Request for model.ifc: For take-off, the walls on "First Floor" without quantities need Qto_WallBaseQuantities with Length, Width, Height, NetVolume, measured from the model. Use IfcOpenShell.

First a look at what the model holds.

```python
import ifcopenshell
import ifcopenshell.util.element
import ifcopenshell.util.unit

model = ifcopenshell.open("model.ifc")
print(model.schema)
for unit_type in ("LENGTHUNIT", "AREAUNIT", "VOLUMEUNIT"):
    print(unit_type, ifcopenshell.util.unit.calculate_unit_scale(model, unit_type))
storey = next(s for s in model.by_type("IfcBuildingStorey") if s.Name == "First Floor")
walls = [e for e in ifcopenshell.util.element.get_decomposition(storey) if e.is_a("IfcWall")]
for e in sorted(walls, key=lambda e: e.id()):
    print(e.id(), e.is_a(), e.Name, list(ifcopenshell.util.element.get_psets(e, qtos_only=True)), sep=" | ")
```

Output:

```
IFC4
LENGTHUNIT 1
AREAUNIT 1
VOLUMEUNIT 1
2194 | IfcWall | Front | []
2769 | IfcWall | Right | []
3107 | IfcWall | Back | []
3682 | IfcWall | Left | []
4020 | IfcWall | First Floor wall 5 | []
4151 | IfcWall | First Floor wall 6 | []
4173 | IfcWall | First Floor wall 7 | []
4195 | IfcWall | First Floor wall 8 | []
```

```python
import ifcopenshell
import ifcopenshell.api.pset
import ifcopenshell.geom
import ifcopenshell.util.element
import ifcopenshell.util.shape
import ifcopenshell.util.unit

model = ifcopenshell.open("model.ifc")
unit_scale = ifcopenshell.util.unit.calculate_unit_scale(model)
volume_scale = ifcopenshell.util.unit.calculate_unit_scale(model, "VOLUMEUNIT")
settings = ifcopenshell.geom.settings()

storey = next(s for s in model.by_type("IfcBuildingStorey") if s.Name == "First Floor")
walls = [e for e in ifcopenshell.util.element.get_decomposition(storey) if e.is_a("IfcWall")]

for e in sorted(walls, key=lambda e: e.id()):
    if ifcopenshell.util.element.get_psets(e, qtos_only=True, should_inherit=False):
        continue
    # Geometry comes back in metres, in the element's own axes.
    shape = ifcopenshell.geom.create_shape(settings, e)
    values = {
        "Length": ifcopenshell.util.shape.get_x(shape.geometry) / unit_scale,
        "Width": ifcopenshell.util.shape.get_y(shape.geometry) / unit_scale,
        "Height": ifcopenshell.util.shape.get_z(shape.geometry) / unit_scale,
        "NetVolume": ifcopenshell.util.shape.get_volume(shape.geometry) / volume_scale,
    }
    qto = ifcopenshell.api.pset.add_qto(model, product=e, name="Qto_WallBaseQuantities")
    ifcopenshell.api.pset.edit_qto(model, qto=qto, properties=values)
    print(e.id(), {k: round(v, 3) for k, v in values.items()})

model.write("model_edited.ifc")
```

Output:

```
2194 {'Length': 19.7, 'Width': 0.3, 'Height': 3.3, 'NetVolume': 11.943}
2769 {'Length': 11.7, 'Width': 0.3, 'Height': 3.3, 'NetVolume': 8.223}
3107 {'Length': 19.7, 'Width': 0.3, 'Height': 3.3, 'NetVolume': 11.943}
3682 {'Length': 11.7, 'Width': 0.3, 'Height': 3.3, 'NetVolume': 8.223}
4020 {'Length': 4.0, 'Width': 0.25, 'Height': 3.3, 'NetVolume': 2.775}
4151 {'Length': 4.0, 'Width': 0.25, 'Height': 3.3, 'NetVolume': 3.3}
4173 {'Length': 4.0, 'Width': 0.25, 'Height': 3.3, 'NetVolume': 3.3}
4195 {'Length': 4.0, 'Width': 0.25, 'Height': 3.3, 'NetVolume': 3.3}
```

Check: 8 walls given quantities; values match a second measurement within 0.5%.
